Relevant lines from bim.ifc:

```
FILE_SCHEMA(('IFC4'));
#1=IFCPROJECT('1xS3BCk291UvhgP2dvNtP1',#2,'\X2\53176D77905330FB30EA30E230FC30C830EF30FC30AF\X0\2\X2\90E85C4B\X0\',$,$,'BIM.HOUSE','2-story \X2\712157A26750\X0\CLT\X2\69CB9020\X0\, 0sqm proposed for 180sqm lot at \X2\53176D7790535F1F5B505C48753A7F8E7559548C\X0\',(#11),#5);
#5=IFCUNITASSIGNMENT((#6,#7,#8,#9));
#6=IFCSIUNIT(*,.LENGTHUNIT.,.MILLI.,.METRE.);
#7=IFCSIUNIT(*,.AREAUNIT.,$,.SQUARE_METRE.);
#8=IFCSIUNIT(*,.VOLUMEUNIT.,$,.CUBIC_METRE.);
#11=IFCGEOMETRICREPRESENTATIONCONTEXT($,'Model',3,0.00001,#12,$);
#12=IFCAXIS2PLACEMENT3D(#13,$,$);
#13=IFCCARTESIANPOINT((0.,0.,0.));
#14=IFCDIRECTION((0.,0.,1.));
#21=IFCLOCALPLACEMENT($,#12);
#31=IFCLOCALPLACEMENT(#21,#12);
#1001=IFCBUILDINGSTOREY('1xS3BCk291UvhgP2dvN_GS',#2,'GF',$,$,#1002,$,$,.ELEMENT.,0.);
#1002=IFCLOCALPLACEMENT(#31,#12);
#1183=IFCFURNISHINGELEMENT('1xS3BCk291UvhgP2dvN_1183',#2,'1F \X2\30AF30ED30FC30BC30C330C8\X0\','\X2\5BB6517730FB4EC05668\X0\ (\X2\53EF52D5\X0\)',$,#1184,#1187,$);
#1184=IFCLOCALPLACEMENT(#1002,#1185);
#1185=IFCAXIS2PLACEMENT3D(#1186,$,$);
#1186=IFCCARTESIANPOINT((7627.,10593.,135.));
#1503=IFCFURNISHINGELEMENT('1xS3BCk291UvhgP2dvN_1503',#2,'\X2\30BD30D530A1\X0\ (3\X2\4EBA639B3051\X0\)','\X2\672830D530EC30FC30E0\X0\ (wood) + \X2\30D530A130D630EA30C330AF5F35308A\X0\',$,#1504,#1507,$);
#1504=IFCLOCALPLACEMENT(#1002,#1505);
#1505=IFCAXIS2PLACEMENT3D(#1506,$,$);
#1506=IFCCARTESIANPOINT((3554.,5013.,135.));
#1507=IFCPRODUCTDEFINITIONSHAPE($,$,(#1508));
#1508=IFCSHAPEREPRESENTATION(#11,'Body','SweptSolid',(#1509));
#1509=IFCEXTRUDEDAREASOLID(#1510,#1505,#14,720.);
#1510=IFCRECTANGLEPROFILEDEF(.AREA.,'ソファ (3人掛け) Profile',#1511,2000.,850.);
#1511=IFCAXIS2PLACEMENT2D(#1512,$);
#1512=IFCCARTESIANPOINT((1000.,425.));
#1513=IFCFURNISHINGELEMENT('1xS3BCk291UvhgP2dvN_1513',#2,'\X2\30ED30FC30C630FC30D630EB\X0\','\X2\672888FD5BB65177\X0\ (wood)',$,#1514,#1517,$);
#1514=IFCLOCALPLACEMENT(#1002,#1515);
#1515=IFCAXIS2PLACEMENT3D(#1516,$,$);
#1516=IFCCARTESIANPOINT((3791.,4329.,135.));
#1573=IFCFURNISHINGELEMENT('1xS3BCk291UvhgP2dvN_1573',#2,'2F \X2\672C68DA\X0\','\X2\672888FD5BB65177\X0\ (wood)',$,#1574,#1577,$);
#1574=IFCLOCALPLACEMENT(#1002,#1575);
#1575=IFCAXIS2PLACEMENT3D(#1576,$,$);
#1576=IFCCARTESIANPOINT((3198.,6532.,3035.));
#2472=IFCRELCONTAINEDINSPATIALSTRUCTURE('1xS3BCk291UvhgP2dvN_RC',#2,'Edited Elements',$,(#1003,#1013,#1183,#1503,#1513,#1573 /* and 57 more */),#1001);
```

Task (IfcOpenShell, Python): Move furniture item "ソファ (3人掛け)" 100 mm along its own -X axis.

```python
import ifcopenshell
import ifcopenshell.api.geometry
import ifcopenshell.util.placement
import ifcopenshell.util.unit

model = ifcopenshell.open("bim.ifc")
unit_scale = ifcopenshell.util.unit.calculate_unit_scale(model)

item = model.by_guid("1xS3BCk291UvhgP2dvN_1503")
matrix = ifcopenshell.util.placement.get_local_placement(item.ObjectPlacement)
matrix[:3, 3] -= matrix[:3, 0] * 0.1 / unit_scale
ifcopenshell.api.geometry.edit_object_placement(model, product=item, matrix=matrix, is_si=False)

print(ifcopenshell.util.placement.get_local_placement(item.ObjectPlacement).round(3) + 0.0)

model.write("bim_v2.ifc")
```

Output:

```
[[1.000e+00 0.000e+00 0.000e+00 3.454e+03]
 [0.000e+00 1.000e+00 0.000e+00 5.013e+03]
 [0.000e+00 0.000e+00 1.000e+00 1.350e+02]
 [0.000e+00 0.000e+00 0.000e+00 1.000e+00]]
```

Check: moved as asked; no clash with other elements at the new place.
